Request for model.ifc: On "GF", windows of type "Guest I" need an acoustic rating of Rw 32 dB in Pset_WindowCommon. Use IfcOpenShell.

First a look at what the model holds.

```python
import ifcopenshell
import ifcopenshell.util.element

model = ifcopenshell.open("model.ifc")
print(model.schema)
storey = next(s for s in model.by_type("IfcBuildingStorey") if s.Name == "GF")
windows = [e for e in ifcopenshell.util.element.get_decomposition(storey) if e.is_a("IfcWindow")]
seen = {}
for e in windows:
    element_type = ifcopenshell.util.element.get_type(e)
    key = (element_type.Name if element_type != e and element_type else None, ifcopenshell.util.element.get_pset(e, "Pset_WindowCommon", "AcousticRating"))
    seen[key] = seen.get(key, 0) + 1
for (name, value), count in sorted(seen.items(), key=str):
    print(count, "x", name, "|", value)
```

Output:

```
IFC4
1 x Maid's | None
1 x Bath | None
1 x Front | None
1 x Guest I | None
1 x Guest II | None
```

```python
import ifcopenshell
import ifcopenshell.api.pset
import ifcopenshell.util.element

model = ifcopenshell.open("model.ifc")

storey = next(s for s in model.by_type("IfcBuildingStorey") if s.Name == "GF")
windows = [e for e in ifcopenshell.util.element.get_decomposition(storey) if e.is_a("IfcWindow")]

count = 0
for e in windows:
    element_type = ifcopenshell.util.element.get_type(e)
    if element_type in (None, e) or element_type.Name != "Guest I":
        continue
    # add_pset returns the element's existing set when there is one.
    pset = ifcopenshell.api.pset.add_pset(model, product=e, name="Pset_WindowCommon")
    ifcopenshell.api.pset.edit_pset(model, pset=pset, properties={"AcousticRating": "Rw 32 dB"})
    count += 1

print(count, "windows updated")

model.write("model_rev.ifc")
```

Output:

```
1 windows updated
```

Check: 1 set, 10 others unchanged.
